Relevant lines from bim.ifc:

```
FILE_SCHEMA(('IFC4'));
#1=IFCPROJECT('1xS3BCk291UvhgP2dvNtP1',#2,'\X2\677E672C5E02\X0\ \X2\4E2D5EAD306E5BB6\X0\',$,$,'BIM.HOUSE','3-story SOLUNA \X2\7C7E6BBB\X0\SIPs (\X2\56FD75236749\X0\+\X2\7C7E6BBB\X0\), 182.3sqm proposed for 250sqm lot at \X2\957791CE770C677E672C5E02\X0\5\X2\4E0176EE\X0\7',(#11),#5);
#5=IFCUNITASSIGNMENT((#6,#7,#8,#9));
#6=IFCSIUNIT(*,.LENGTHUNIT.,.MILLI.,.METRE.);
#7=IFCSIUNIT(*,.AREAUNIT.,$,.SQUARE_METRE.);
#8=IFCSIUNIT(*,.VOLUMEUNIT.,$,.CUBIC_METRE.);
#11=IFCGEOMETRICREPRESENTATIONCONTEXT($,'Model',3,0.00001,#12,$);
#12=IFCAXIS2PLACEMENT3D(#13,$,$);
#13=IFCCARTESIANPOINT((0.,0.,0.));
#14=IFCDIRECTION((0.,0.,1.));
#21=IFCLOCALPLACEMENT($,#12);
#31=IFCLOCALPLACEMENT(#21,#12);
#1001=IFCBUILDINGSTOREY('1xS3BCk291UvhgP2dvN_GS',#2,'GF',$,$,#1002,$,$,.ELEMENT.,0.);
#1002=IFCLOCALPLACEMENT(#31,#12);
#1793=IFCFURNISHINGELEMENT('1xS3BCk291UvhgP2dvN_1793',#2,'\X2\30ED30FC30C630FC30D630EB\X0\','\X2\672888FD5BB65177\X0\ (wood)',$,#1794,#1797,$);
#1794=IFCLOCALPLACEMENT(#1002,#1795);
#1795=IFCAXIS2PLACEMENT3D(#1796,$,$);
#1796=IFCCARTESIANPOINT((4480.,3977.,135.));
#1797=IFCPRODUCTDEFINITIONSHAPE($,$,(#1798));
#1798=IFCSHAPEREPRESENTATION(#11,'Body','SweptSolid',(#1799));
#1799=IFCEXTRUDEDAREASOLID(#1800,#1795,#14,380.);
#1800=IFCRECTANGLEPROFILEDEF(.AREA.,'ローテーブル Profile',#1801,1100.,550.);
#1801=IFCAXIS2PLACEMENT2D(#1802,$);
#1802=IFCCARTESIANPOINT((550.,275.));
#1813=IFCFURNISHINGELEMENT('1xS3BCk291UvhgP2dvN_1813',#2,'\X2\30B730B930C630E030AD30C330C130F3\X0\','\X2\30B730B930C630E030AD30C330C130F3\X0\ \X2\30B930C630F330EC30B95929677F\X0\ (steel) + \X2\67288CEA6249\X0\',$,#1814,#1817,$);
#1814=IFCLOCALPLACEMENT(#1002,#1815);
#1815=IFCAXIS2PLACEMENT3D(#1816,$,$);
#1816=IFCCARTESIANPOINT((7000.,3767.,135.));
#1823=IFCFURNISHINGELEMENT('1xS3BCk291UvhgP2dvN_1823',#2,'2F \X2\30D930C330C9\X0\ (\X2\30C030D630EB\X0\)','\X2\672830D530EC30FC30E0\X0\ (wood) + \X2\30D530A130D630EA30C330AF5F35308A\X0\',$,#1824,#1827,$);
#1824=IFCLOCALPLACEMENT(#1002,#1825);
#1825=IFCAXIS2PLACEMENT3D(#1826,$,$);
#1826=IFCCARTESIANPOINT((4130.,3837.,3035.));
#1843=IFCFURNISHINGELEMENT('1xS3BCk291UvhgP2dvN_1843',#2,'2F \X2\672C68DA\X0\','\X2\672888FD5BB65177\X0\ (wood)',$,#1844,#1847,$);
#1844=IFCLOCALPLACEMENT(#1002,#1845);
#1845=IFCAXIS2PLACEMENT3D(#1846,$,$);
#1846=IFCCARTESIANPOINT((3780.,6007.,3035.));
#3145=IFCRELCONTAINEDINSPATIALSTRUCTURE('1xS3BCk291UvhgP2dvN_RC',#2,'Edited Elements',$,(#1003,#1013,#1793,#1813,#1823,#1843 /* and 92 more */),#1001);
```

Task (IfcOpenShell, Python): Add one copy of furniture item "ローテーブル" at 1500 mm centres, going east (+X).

```python
import numpy as np
import ifcopenshell
import ifcopenshell.api.geometry
import ifcopenshell.api.root
import ifcopenshell.util.element
import ifcopenshell.util.placement

model = ifcopenshell.open("bim.ifc")


def reuse_history(source, copy):
    """copy_class also copies each property set's owner history, people and application; keep the originals."""
    for rel in copy.IsDefinedBy:
        if rel.is_a("IfcRelDefinesByProperties") and (history := rel.RelatingPropertyDefinition.OwnerHistory):
            rel.RelatingPropertyDefinition.OwnerHistory = source.OwnerHistory
            ifcopenshell.util.element.remove_deep2(model, history)


source = model.by_id(1793)
base = ifcopenshell.util.placement.get_local_placement(source.ObjectPlacement)
step = np.array([1.0, 0.0, 0.0]) * 1500.0

for i in range(1, 2):
    copy = ifcopenshell.api.root.copy_class(model, product=source)
    copy.Representation = ifcopenshell.util.element.copy_deep(
        model, source.Representation, exclude=["IfcGeometricRepresentationContext", "IfcRepresentationMap"]
    )
    reuse_history(source, copy)
    matrix = base.copy()
    matrix[:3, 3] += i * step
    print("added at", matrix[:3, 3].round(3) + 0.0)
    ifcopenshell.api.geometry.edit_object_placement(model, product=copy, matrix=matrix, is_si=False)

model.write("bim_edited.ifc")
```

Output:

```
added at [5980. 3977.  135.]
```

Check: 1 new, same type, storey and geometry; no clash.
